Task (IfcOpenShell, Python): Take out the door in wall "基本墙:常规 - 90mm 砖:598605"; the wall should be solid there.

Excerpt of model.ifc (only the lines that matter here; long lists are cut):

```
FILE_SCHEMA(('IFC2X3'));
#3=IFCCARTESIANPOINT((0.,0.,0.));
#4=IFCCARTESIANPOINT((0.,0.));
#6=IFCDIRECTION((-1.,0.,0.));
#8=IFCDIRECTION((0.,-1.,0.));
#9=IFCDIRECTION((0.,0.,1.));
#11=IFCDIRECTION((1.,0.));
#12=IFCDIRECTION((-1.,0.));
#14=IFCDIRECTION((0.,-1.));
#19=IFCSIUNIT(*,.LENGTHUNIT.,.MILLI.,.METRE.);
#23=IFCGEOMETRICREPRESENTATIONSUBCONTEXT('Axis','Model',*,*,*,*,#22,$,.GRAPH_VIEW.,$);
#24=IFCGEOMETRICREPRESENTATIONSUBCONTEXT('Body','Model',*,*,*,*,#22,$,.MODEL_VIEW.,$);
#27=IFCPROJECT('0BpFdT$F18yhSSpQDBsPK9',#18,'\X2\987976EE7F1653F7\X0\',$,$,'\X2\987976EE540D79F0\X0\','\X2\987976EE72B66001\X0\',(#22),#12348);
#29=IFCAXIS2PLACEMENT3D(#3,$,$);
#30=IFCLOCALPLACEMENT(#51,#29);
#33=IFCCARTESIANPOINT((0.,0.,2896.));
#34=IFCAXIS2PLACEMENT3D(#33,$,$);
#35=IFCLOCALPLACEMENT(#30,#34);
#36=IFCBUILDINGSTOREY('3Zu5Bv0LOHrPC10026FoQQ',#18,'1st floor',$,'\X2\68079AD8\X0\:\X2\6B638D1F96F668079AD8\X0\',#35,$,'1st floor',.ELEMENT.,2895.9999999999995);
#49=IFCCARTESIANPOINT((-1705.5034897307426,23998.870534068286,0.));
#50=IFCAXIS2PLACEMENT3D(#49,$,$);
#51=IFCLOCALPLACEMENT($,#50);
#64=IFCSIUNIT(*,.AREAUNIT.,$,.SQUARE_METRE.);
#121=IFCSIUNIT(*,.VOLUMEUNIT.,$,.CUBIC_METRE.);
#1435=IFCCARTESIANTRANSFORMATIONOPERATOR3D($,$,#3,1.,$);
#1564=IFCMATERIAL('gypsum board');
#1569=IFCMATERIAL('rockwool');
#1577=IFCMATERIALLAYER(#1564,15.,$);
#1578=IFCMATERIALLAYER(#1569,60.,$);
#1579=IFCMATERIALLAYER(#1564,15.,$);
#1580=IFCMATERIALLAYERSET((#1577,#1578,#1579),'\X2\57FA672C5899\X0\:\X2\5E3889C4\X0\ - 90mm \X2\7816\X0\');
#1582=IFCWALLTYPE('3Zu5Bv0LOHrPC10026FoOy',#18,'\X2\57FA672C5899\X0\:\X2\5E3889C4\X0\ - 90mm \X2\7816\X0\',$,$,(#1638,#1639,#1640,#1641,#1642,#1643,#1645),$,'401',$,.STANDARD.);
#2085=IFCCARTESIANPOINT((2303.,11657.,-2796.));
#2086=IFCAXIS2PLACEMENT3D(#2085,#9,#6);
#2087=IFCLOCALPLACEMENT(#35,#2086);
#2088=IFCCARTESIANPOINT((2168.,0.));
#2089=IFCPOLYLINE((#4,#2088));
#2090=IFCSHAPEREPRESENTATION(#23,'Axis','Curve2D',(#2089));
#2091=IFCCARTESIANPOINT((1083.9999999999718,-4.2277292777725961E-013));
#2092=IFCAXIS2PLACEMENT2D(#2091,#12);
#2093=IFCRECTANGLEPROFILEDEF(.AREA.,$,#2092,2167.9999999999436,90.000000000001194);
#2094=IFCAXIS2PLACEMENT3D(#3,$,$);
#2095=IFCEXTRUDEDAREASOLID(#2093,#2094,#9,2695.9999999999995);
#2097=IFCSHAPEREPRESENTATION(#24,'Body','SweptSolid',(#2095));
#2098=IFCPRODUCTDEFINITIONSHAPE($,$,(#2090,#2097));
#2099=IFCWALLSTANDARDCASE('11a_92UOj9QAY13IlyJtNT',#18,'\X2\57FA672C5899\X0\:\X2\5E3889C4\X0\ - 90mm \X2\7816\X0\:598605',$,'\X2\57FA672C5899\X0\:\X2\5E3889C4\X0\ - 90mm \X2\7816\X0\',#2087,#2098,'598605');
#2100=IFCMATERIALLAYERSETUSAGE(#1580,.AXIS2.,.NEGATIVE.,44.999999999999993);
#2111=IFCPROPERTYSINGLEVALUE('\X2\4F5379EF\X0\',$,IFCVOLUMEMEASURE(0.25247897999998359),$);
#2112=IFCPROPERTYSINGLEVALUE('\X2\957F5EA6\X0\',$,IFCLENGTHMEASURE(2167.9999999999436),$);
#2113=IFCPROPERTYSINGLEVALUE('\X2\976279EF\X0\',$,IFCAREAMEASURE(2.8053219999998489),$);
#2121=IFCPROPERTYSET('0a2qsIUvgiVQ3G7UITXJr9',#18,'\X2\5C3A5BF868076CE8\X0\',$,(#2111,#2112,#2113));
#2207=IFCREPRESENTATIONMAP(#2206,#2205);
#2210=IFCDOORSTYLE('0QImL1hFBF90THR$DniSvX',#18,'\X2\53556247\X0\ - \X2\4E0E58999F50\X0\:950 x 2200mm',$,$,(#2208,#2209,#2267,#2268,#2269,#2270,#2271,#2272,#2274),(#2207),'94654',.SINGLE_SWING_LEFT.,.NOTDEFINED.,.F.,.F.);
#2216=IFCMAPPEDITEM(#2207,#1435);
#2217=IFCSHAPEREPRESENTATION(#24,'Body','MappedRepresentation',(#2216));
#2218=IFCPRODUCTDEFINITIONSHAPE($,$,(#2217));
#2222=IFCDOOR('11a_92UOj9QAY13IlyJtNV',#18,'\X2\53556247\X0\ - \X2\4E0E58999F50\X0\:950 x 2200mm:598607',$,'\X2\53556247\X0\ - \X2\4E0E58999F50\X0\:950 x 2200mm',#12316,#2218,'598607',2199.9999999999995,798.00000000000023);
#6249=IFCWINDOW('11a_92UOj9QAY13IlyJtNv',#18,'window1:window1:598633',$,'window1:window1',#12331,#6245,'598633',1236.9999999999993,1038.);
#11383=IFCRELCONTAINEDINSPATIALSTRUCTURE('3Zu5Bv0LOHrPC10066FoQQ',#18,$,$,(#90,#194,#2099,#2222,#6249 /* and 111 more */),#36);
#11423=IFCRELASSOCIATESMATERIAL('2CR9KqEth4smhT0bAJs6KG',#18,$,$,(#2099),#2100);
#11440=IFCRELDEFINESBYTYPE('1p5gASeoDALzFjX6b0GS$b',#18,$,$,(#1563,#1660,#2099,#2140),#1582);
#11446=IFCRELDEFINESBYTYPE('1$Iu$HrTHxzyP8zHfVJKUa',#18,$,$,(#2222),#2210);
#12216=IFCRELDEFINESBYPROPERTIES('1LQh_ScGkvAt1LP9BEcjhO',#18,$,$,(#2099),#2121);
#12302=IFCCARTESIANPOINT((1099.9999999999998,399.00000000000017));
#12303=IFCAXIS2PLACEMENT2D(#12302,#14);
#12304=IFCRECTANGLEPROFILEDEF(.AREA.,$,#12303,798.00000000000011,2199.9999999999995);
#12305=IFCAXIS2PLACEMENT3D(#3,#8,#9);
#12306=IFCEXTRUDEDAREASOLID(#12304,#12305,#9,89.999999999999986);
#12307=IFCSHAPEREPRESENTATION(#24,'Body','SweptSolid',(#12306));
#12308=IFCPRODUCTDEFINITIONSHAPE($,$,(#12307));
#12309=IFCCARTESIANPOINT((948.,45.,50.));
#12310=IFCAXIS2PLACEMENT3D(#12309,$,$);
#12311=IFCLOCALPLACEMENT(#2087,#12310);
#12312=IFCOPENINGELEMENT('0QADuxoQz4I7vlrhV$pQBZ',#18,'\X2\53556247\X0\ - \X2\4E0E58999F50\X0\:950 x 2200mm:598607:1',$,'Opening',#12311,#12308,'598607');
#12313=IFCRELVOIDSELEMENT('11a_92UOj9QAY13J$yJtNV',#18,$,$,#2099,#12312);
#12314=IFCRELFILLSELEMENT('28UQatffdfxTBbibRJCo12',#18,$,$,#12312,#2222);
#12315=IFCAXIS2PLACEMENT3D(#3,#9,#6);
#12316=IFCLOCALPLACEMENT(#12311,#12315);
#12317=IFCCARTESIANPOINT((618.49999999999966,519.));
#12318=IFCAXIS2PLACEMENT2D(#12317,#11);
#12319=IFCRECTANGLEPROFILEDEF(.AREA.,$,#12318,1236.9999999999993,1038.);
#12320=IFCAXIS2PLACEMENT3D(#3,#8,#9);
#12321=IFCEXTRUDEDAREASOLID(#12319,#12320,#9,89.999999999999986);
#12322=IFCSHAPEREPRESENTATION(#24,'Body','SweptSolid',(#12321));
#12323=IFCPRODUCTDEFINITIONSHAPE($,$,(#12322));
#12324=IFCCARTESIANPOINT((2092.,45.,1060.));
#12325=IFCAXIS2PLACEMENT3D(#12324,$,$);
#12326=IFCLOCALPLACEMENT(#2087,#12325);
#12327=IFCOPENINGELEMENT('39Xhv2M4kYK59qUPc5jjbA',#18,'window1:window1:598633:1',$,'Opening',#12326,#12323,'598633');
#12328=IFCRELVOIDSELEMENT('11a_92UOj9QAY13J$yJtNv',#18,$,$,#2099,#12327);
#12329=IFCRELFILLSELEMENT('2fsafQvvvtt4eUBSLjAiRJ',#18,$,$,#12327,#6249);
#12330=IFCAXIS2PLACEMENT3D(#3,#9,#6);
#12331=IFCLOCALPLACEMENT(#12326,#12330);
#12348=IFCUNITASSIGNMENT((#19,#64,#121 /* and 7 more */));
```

```python
import ifcopenshell
import ifcopenshell.api.feature
import ifcopenshell.api.pset
import ifcopenshell.api.root
import ifcopenshell.geom
import ifcopenshell.util.element
import ifcopenshell.util.shape
import ifcopenshell.util.unit

model = ifcopenshell.open("model.ifc")
area_scale = ifcopenshell.util.unit.calculate_unit_scale(model, "AREAUNIT")
volume_scale = ifcopenshell.util.unit.calculate_unit_scale(model, "VOLUMEUNIT")
settings = ifcopenshell.geom.settings()


def volume(element):
    """Net volume in cubic metres, openings subtracted."""
    shape = ifcopenshell.geom.create_shape(settings, element)
    return ifcopenshell.util.shape.get_volume(shape.geometry)


door = model.by_guid("11a_92UOj9QAY13IlyJtNV")
opening = door.FillsVoids[0].RelatingOpeningElement
wall = opening.VoidsElements[0].RelatingBuildingElement
before = volume(wall)

ifcopenshell.api.root.remove_product(model, product=door)
ifcopenshell.api.feature.remove_feature(model, feature=opening)

after = volume(wall)
thickness = 0.09  # wall thickness in metres

# Update the wall's stored quantities.
pset = model.by_id(ifcopenshell.util.element.get_pset(wall, "尺寸标注", should_inherit=False)["id"])
ifcopenshell.api.pset.edit_pset(model, pset=pset, properties={
    "体积": model.create_entity("IfcVolumeMeasure", after / volume_scale),
    "面积": model.create_entity("IfcAreaMeasure", after / thickness / area_scale),
})

print(f"wall volume {before:.3f} -> {after:.3f} m3")

model.write("model_v2.ifc")
```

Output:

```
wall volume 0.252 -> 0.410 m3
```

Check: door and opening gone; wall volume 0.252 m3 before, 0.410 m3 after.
